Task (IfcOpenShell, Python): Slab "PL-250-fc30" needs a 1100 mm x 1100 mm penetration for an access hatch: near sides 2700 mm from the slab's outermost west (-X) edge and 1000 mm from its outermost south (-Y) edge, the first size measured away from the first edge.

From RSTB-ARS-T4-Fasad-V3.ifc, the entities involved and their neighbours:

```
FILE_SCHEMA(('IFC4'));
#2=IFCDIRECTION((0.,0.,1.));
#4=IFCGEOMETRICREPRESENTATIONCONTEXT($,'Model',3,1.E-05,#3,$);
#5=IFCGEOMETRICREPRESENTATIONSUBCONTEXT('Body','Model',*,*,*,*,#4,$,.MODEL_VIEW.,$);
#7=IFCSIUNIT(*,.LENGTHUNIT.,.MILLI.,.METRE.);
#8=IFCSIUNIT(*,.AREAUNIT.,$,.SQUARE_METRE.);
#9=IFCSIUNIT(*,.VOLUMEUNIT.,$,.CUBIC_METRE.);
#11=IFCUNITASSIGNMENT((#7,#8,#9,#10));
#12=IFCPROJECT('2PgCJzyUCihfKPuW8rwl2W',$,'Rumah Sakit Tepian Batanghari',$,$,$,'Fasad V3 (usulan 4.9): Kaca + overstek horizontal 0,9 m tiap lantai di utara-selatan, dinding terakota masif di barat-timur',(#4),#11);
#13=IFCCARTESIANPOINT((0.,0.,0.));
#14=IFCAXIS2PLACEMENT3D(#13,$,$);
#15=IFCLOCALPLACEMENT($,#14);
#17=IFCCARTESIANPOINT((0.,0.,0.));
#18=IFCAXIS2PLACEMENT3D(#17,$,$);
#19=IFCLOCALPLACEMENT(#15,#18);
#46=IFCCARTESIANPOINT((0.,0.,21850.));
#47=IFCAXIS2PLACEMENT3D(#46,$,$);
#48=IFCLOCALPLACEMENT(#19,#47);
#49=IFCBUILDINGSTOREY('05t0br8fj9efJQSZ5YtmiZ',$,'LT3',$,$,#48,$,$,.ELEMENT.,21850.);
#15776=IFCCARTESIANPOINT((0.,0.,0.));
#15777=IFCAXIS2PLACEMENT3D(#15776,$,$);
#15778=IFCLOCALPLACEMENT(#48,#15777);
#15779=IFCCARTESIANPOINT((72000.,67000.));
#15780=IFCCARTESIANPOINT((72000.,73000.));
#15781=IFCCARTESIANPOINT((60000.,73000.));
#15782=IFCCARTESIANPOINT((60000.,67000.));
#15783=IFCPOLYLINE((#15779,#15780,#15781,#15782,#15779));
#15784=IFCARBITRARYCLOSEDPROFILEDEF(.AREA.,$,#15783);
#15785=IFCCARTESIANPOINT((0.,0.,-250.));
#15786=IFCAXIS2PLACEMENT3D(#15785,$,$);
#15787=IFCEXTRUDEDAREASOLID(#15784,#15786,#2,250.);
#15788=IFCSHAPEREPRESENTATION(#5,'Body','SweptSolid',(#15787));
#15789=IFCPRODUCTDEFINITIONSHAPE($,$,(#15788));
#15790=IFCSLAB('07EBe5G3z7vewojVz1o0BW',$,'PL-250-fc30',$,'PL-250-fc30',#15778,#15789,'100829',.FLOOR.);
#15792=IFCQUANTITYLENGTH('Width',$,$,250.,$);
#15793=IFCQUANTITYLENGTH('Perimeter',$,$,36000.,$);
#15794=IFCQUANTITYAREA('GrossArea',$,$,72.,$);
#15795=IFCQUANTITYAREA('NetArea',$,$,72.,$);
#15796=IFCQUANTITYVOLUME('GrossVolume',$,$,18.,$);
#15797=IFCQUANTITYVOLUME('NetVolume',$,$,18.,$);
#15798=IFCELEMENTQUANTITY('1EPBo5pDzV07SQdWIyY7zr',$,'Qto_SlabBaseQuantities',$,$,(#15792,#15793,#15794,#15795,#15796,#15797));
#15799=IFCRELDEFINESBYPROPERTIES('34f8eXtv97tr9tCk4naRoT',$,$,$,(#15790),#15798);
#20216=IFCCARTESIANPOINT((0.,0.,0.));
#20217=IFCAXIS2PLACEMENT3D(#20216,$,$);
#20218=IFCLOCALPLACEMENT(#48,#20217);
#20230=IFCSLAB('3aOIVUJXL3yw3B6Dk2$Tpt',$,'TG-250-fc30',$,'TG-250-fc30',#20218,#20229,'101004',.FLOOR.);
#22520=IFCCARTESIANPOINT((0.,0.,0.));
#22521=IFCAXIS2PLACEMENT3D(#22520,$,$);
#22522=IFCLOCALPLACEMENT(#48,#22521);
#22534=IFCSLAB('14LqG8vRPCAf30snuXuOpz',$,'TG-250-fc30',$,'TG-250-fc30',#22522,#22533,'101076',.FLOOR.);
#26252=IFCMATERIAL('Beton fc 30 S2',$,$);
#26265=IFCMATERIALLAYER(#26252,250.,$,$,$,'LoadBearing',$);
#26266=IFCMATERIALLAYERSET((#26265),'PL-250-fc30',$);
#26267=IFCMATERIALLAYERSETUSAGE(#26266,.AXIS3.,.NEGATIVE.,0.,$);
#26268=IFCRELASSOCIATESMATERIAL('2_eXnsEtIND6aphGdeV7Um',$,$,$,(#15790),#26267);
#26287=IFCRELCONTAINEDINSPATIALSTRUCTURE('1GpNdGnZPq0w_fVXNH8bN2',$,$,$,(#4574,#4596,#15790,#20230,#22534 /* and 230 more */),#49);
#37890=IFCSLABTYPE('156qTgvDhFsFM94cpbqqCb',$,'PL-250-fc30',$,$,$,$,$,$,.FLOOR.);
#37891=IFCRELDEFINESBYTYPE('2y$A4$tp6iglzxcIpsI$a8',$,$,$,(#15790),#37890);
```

```python
import numpy as np
import ifcopenshell
import ifcopenshell.api.feature
import ifcopenshell.api.geometry
import ifcopenshell.api.pset
import ifcopenshell.api.root
import ifcopenshell.geom
import ifcopenshell.util.element
import ifcopenshell.util.placement
import ifcopenshell.util.representation
import ifcopenshell.util.shape
import ifcopenshell.util.unit

model = ifcopenshell.open("RSTB-ARS-T4-Fasad-V3.ifc")
unit_scale = ifcopenshell.util.unit.calculate_unit_scale(model)
area_scale = ifcopenshell.util.unit.calculate_unit_scale(model, "AREAUNIT")
volume_scale = ifcopenshell.util.unit.calculate_unit_scale(model, "VOLUMEUNIT")
settings = ifcopenshell.geom.settings()


def volume(element):
    """Net volume in cubic metres, openings subtracted."""
    shape = ifcopenshell.geom.create_shape(settings, element)
    return ifcopenshell.util.shape.get_volume(shape.geometry)


slab = model.by_guid("07EBe5G3z7vewojVz1o0BW")
before = volume(slab)

# Extent in the slab's own axes, in metres. The edges named are its -X and -Y sides.
slab_shape = ifcopenshell.geom.create_shape(settings, slab)
vertices = ifcopenshell.util.shape.get_vertices(slab_shape.geometry)
x_min, y_min, bottom = vertices.min(axis=0)
top = vertices[:, 2].max()

opening = ifcopenshell.api.root.create_entity(model, ifc_class="IfcOpeningElement", name="Access hatch opening", predefined_type="OPENING")
context = ifcopenshell.util.representation.get_context(model, "Model", "Body", "MODEL_VIEW")
width, depth = 1.1, 1.1
outline = [(0.0, 0.0), (width, 0.0), (width, depth), (0.0, depth), (0.0, 0.0)]
# Overshoot both faces by 50 mm so the cut is clean.
shape = ifcopenshell.api.geometry.add_slab_representation(
    model, context=context, depth=top - bottom + 0.1, polyline=outline
)
ifcopenshell.api.geometry.assign_representation(model, product=opening, representation=shape)

matrix = ifcopenshell.util.placement.get_local_placement(slab.ObjectPlacement)
matrix[:, 3] = matrix @ np.append(np.array([x_min + 2.7, y_min + 1, bottom - 0.05]) / unit_scale, 1.0)
ifcopenshell.api.geometry.edit_object_placement(model, product=opening, matrix=matrix, is_si=False)
ifcopenshell.api.feature.add_feature(model, feature=opening, element=slab)

after = volume(slab)

# Update the slab's stored quantities.
qto = model.by_id(ifcopenshell.util.element.get_pset(slab, "Qto_SlabBaseQuantities", should_inherit=False)["id"])
ifcopenshell.api.pset.edit_qto(model, qto=qto, properties={
    "NetArea": after / (top - bottom) / area_scale,
    "NetVolume": after / volume_scale,
})

print(f"slab volume {before:.3f} -> {after:.3f} m3")

model.write("RSTB-ARS-T4-Fasad-V3_updated.ifc")
```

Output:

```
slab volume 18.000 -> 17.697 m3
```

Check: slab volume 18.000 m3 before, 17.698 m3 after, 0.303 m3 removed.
